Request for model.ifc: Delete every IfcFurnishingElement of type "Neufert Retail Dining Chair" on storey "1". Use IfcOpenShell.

First a look at what the model holds.

```python
import ifcopenshell
import ifcopenshell.util.element

model = ifcopenshell.open("model.ifc")
print(model.schema)
storey = next(s for s in model.by_type("IfcBuildingStorey") if s.Name == "1")
furniture = [e for e in ifcopenshell.util.element.get_decomposition(storey) if e.is_a("IfcFurnishingElement")]
seen = {}
for e in furniture:
    element_type = ifcopenshell.util.element.get_type(e)
    name = element_type.Name if element_type not in (None, e) else None
    seen[name] = seen.get(name, 0) + 1
for name, count in sorted(seen.items(), key=str):
    print(count, "x", name)
```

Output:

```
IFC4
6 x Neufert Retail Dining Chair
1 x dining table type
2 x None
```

```python
import ifcopenshell
import ifcopenshell.api.root
import ifcopenshell.util.element

model = ifcopenshell.open("model.ifc")

storey = next(s for s in model.by_type("IfcBuildingStorey") if s.Name == "1")
furniture = [e for e in ifcopenshell.util.element.get_decomposition(storey) if e.is_a("IfcFurnishingElement")]
targets = [e for e in furniture if (t := ifcopenshell.util.element.get_type(e)) not in (None, e) and t.Name == "Neufert Retail Dining Chair"]

for e in targets:
    ifcopenshell.api.root.remove_product(model, product=e)
print(len(targets), "removed")

model.write("model-out.ifc")
```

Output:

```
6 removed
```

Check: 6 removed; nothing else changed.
